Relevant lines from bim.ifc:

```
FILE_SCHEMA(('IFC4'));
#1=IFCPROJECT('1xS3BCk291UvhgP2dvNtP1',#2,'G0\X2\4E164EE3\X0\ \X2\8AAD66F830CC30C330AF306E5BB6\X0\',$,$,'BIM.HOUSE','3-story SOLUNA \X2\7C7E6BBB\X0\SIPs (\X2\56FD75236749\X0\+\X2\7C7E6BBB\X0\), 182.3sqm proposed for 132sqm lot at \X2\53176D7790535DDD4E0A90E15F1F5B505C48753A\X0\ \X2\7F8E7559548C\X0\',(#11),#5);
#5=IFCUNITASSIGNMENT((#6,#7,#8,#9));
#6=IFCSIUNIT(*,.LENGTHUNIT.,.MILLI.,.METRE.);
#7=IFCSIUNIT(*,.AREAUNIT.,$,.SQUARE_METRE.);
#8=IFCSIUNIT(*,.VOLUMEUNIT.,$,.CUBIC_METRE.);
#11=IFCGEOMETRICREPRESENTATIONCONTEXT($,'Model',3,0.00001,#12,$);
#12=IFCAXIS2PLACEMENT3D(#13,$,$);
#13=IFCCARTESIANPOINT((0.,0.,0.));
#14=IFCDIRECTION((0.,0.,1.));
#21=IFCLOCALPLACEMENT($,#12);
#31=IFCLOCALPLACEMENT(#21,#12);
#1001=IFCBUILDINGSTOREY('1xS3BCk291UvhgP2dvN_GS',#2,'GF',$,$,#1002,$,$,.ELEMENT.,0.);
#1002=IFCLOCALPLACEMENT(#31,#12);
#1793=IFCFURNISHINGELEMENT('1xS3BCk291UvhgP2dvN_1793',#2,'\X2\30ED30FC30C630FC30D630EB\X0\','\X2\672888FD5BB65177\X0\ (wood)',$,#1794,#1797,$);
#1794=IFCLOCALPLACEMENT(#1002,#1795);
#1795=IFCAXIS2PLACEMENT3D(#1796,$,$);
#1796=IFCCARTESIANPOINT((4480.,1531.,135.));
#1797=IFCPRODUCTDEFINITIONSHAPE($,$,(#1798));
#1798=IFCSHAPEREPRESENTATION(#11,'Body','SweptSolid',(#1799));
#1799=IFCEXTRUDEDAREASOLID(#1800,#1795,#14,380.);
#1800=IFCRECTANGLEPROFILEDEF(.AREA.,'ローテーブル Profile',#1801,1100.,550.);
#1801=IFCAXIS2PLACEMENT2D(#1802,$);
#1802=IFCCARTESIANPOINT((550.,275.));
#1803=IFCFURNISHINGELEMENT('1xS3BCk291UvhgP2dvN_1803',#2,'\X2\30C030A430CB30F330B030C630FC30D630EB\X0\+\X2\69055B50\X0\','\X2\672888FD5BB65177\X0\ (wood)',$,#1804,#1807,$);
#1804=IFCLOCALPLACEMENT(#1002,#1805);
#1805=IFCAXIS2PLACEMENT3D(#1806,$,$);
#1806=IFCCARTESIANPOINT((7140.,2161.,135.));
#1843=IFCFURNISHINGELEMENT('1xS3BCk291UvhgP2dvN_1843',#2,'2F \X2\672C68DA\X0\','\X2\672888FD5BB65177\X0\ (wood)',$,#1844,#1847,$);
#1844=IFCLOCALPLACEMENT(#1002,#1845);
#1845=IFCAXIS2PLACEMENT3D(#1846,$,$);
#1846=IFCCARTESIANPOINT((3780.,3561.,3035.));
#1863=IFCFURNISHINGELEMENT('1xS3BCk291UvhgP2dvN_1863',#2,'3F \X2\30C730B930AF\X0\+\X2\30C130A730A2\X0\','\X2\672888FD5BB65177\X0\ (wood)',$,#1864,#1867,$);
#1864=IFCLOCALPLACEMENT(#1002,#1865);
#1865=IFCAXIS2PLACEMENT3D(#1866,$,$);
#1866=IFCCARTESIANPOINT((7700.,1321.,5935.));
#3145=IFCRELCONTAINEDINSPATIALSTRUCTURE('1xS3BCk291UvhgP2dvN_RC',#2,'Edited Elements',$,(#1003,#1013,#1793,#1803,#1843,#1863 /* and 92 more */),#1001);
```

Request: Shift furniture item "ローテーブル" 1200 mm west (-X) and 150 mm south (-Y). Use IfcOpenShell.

```python
import ifcopenshell
import ifcopenshell.api.geometry
import ifcopenshell.util.placement

model = ifcopenshell.open("bim.ifc")

item = model.by_id(1793)
matrix = ifcopenshell.util.placement.get_local_placement(item.ObjectPlacement)
matrix[0, 3] -= 1200.0
matrix[1, 3] -= 150.0
ifcopenshell.api.geometry.edit_object_placement(model, product=item, matrix=matrix, is_si=False)

print(ifcopenshell.util.placement.get_local_placement(item.ObjectPlacement).round(3) + 0.0)

model.write("bim-out.ifc")
```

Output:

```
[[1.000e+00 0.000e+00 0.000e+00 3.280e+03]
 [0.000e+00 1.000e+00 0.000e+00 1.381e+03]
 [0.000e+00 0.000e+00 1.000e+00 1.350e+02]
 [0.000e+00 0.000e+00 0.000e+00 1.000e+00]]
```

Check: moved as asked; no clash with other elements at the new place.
